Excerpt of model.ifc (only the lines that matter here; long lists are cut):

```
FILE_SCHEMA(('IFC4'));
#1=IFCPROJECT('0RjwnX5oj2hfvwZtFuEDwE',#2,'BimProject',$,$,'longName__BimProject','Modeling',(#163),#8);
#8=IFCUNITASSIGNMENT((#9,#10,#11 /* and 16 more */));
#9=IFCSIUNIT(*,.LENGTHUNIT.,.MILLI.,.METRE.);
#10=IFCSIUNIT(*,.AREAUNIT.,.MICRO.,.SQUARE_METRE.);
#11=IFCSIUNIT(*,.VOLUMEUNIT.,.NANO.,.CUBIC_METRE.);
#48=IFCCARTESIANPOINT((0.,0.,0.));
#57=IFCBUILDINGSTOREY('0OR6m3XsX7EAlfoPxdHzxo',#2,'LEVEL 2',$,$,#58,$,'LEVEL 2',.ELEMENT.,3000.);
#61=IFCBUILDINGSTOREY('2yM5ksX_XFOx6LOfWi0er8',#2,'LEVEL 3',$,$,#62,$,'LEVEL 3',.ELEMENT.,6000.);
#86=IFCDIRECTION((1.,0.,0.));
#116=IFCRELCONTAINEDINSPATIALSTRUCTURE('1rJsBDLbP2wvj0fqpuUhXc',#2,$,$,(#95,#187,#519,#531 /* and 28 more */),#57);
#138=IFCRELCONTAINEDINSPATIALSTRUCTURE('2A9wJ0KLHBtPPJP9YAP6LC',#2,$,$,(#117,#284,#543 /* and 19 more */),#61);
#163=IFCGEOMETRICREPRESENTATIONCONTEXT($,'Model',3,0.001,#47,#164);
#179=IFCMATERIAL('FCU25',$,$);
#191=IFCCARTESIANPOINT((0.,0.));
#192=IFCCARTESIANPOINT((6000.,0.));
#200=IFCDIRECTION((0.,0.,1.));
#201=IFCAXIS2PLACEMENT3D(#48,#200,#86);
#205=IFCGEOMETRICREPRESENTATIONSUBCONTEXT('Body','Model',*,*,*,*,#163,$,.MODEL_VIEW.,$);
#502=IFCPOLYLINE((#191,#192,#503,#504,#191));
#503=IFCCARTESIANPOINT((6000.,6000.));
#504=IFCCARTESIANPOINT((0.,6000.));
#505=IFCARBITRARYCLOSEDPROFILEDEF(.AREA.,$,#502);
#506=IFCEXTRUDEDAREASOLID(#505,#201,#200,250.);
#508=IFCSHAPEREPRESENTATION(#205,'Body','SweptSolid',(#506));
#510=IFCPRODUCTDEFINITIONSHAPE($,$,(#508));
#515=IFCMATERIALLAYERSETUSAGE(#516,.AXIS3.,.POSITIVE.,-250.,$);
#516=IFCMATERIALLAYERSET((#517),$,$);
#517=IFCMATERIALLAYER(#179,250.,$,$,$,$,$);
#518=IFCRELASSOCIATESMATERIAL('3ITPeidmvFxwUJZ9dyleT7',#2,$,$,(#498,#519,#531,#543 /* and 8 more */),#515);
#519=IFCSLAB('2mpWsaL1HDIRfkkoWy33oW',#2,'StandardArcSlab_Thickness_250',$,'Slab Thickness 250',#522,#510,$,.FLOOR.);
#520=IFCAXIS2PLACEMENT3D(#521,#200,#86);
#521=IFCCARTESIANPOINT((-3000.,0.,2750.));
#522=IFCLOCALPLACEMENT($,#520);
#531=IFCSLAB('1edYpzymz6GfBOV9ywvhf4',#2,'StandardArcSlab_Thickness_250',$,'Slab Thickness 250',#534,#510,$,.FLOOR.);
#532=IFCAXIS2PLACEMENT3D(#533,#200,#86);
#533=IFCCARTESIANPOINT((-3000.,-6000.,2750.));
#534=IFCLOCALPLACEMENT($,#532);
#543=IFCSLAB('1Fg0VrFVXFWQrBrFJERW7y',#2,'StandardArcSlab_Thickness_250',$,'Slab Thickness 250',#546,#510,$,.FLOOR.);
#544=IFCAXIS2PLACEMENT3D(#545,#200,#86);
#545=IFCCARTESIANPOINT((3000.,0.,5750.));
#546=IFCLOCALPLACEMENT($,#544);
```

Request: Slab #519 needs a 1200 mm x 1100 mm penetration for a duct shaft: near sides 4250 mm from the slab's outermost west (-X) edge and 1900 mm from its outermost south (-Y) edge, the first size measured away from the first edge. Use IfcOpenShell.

```python
import numpy as np
import ifcopenshell
import ifcopenshell.api.feature
import ifcopenshell.api.geometry
import ifcopenshell.api.root
import ifcopenshell.geom
import ifcopenshell.util.placement
import ifcopenshell.util.representation
import ifcopenshell.util.shape
import ifcopenshell.util.unit

model = ifcopenshell.open("model.ifc")
unit_scale = ifcopenshell.util.unit.calculate_unit_scale(model)
settings = ifcopenshell.geom.settings()


def volume(element):
    """Net volume in cubic metres, openings subtracted."""
    shape = ifcopenshell.geom.create_shape(settings, element)
    return ifcopenshell.util.shape.get_volume(shape.geometry)


slab = model.by_id(519)
before = volume(slab)

# Extent in the slab's own axes, in metres. The edges named are its -X and -Y sides.
slab_shape = ifcopenshell.geom.create_shape(settings, slab)
vertices = ifcopenshell.util.shape.get_vertices(slab_shape.geometry)
x_min, y_min, bottom = vertices.min(axis=0)
top = vertices[:, 2].max()

opening = ifcopenshell.api.root.create_entity(model, ifc_class="IfcOpeningElement", name="Duct shaft opening", predefined_type="OPENING")
context = ifcopenshell.util.representation.get_context(model, "Model", "Body", "MODEL_VIEW")
width, depth = 1.2, 1.1
outline = [(0.0, 0.0), (width, 0.0), (width, depth), (0.0, depth), (0.0, 0.0)]
# Overshoot both faces by 50 mm so the cut is clean.
shape = ifcopenshell.api.geometry.add_slab_representation(
    model, context=context, depth=top - bottom + 0.1, polyline=outline
)
ifcopenshell.api.geometry.assign_representation(model, product=opening, representation=shape)

matrix = ifcopenshell.util.placement.get_local_placement(slab.ObjectPlacement)
matrix[:, 3] = matrix @ np.append(np.array([x_min + 4.25, y_min + 1.9, bottom - 0.05]) / unit_scale, 1.0)
ifcopenshell.api.geometry.edit_object_placement(model, product=opening, matrix=matrix, is_si=False)
ifcopenshell.api.feature.add_feature(model, feature=opening, element=slab)

after = volume(slab)

print(f"slab volume {before:.3f} -> {after:.3f} m3")

model.write("model-out.ifc")
```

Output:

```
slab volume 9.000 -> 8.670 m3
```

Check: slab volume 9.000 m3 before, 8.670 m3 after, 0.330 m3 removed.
